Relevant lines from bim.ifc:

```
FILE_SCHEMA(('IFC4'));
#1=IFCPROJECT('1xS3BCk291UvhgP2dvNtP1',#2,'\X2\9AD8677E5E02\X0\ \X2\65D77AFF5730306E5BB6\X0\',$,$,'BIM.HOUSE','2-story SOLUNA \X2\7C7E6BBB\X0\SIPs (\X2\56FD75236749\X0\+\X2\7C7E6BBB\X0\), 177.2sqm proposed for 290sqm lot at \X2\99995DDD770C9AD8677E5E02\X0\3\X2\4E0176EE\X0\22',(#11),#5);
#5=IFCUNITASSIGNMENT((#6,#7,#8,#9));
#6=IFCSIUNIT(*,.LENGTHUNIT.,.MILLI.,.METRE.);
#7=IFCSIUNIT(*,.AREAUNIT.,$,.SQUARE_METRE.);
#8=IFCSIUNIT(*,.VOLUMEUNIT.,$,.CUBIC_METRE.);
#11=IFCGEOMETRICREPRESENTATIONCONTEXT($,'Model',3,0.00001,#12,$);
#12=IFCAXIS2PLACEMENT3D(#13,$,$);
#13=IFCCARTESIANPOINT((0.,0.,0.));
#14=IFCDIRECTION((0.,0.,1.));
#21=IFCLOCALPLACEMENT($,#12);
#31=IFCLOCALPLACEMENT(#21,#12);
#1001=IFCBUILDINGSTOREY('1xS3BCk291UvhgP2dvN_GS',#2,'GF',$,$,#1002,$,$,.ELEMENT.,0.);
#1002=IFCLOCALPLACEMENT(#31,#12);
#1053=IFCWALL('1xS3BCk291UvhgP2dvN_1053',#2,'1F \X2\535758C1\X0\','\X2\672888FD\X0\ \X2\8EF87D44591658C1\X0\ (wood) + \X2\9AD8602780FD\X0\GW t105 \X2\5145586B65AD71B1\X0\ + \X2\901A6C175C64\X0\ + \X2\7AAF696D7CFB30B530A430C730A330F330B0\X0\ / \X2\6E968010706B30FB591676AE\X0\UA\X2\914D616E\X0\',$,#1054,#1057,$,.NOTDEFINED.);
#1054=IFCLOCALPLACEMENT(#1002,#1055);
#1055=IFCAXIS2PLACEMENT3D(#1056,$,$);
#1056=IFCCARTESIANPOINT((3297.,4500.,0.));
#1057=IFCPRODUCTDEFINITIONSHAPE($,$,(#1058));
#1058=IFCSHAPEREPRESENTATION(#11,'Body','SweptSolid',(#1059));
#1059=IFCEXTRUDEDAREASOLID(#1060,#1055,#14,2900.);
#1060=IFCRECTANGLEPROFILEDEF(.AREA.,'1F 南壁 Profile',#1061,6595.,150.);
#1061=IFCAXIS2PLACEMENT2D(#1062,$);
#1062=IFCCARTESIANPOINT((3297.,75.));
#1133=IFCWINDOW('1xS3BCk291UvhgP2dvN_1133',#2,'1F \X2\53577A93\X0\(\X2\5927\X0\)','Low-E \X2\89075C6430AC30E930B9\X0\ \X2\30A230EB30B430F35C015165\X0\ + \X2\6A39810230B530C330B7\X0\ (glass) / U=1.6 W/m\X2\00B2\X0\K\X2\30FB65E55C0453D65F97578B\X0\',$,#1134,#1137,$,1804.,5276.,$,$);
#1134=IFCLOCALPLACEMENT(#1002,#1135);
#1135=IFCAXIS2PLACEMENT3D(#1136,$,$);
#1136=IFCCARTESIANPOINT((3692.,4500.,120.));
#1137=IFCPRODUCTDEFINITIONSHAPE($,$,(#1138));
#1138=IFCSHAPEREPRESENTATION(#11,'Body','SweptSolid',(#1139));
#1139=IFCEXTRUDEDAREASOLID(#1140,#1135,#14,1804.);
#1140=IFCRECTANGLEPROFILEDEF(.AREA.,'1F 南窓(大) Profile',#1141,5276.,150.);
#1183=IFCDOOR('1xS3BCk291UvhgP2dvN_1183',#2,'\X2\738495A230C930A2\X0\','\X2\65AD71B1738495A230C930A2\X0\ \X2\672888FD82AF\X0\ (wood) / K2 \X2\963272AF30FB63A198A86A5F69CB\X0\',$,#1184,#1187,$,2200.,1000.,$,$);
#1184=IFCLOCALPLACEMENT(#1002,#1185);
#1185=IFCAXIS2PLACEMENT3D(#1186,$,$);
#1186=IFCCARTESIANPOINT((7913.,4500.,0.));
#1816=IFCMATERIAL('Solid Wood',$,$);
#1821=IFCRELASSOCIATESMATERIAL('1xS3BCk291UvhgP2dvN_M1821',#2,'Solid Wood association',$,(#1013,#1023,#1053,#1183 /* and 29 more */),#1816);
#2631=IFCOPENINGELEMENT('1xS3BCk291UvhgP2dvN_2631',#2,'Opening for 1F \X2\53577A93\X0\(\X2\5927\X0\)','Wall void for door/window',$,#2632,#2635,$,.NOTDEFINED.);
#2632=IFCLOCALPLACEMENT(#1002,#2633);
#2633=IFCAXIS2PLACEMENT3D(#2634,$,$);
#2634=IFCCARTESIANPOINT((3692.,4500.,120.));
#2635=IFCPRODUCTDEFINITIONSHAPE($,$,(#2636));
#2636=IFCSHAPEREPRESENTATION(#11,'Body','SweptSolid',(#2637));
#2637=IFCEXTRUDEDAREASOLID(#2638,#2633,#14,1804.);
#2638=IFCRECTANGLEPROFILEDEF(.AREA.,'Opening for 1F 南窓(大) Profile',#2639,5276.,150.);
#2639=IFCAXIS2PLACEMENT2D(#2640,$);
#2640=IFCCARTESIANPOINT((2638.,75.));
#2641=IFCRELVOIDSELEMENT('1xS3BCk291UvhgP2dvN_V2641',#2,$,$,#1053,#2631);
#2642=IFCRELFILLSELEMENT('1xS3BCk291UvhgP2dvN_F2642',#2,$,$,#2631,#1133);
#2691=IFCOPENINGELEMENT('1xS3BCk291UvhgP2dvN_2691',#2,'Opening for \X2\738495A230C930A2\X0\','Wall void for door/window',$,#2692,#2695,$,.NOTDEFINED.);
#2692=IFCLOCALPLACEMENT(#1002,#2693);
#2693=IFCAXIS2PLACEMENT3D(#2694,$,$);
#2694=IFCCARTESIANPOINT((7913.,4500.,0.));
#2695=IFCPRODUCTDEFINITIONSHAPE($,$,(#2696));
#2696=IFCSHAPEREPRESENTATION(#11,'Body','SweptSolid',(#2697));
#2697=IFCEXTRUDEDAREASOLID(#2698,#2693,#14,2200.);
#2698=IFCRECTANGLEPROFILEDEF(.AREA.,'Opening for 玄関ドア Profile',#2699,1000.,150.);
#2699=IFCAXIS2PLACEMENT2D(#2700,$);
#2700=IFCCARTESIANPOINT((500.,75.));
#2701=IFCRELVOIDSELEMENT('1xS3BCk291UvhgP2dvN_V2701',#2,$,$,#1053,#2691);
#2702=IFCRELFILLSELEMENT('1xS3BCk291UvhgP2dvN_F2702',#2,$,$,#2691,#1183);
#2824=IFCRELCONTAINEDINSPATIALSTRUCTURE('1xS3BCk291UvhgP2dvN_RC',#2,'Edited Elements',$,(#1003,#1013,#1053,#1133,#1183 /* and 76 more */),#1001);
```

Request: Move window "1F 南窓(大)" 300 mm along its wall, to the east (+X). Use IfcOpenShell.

```python
import ifcopenshell
import ifcopenshell.api.geometry
import ifcopenshell.util.placement
import ifcopenshell.util.unit

model = ifcopenshell.open("bim.ifc")
unit_scale = ifcopenshell.util.unit.calculate_unit_scale(model)

window = model.by_id(1133)
opening = window.FillsVoids[0].RelatingOpeningElement
wall = opening.VoidsElements[0].RelatingBuildingElement

wall_matrix = ifcopenshell.util.placement.get_local_placement(wall.ObjectPlacement)
shift = wall_matrix[:3, 0] * 0.3 / unit_scale
before = ifcopenshell.util.placement.get_local_placement(window.ObjectPlacement)[:3, 3].copy()

# The window is not placed relative to its opening, so move both.
for product in (opening, window):
    matrix = ifcopenshell.util.placement.get_local_placement(product.ObjectPlacement)
    matrix[:3, 3] += shift
    ifcopenshell.api.geometry.edit_object_placement(model, product=product, matrix=matrix, is_si=False)

after = ifcopenshell.util.placement.get_local_placement(window.ObjectPlacement)[:3, 3]
print("window moved by", (after - before).round(3) + 0.0)

model.write("bim_edited.ifc")
```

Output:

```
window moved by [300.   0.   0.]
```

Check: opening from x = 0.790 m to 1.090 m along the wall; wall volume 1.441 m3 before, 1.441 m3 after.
